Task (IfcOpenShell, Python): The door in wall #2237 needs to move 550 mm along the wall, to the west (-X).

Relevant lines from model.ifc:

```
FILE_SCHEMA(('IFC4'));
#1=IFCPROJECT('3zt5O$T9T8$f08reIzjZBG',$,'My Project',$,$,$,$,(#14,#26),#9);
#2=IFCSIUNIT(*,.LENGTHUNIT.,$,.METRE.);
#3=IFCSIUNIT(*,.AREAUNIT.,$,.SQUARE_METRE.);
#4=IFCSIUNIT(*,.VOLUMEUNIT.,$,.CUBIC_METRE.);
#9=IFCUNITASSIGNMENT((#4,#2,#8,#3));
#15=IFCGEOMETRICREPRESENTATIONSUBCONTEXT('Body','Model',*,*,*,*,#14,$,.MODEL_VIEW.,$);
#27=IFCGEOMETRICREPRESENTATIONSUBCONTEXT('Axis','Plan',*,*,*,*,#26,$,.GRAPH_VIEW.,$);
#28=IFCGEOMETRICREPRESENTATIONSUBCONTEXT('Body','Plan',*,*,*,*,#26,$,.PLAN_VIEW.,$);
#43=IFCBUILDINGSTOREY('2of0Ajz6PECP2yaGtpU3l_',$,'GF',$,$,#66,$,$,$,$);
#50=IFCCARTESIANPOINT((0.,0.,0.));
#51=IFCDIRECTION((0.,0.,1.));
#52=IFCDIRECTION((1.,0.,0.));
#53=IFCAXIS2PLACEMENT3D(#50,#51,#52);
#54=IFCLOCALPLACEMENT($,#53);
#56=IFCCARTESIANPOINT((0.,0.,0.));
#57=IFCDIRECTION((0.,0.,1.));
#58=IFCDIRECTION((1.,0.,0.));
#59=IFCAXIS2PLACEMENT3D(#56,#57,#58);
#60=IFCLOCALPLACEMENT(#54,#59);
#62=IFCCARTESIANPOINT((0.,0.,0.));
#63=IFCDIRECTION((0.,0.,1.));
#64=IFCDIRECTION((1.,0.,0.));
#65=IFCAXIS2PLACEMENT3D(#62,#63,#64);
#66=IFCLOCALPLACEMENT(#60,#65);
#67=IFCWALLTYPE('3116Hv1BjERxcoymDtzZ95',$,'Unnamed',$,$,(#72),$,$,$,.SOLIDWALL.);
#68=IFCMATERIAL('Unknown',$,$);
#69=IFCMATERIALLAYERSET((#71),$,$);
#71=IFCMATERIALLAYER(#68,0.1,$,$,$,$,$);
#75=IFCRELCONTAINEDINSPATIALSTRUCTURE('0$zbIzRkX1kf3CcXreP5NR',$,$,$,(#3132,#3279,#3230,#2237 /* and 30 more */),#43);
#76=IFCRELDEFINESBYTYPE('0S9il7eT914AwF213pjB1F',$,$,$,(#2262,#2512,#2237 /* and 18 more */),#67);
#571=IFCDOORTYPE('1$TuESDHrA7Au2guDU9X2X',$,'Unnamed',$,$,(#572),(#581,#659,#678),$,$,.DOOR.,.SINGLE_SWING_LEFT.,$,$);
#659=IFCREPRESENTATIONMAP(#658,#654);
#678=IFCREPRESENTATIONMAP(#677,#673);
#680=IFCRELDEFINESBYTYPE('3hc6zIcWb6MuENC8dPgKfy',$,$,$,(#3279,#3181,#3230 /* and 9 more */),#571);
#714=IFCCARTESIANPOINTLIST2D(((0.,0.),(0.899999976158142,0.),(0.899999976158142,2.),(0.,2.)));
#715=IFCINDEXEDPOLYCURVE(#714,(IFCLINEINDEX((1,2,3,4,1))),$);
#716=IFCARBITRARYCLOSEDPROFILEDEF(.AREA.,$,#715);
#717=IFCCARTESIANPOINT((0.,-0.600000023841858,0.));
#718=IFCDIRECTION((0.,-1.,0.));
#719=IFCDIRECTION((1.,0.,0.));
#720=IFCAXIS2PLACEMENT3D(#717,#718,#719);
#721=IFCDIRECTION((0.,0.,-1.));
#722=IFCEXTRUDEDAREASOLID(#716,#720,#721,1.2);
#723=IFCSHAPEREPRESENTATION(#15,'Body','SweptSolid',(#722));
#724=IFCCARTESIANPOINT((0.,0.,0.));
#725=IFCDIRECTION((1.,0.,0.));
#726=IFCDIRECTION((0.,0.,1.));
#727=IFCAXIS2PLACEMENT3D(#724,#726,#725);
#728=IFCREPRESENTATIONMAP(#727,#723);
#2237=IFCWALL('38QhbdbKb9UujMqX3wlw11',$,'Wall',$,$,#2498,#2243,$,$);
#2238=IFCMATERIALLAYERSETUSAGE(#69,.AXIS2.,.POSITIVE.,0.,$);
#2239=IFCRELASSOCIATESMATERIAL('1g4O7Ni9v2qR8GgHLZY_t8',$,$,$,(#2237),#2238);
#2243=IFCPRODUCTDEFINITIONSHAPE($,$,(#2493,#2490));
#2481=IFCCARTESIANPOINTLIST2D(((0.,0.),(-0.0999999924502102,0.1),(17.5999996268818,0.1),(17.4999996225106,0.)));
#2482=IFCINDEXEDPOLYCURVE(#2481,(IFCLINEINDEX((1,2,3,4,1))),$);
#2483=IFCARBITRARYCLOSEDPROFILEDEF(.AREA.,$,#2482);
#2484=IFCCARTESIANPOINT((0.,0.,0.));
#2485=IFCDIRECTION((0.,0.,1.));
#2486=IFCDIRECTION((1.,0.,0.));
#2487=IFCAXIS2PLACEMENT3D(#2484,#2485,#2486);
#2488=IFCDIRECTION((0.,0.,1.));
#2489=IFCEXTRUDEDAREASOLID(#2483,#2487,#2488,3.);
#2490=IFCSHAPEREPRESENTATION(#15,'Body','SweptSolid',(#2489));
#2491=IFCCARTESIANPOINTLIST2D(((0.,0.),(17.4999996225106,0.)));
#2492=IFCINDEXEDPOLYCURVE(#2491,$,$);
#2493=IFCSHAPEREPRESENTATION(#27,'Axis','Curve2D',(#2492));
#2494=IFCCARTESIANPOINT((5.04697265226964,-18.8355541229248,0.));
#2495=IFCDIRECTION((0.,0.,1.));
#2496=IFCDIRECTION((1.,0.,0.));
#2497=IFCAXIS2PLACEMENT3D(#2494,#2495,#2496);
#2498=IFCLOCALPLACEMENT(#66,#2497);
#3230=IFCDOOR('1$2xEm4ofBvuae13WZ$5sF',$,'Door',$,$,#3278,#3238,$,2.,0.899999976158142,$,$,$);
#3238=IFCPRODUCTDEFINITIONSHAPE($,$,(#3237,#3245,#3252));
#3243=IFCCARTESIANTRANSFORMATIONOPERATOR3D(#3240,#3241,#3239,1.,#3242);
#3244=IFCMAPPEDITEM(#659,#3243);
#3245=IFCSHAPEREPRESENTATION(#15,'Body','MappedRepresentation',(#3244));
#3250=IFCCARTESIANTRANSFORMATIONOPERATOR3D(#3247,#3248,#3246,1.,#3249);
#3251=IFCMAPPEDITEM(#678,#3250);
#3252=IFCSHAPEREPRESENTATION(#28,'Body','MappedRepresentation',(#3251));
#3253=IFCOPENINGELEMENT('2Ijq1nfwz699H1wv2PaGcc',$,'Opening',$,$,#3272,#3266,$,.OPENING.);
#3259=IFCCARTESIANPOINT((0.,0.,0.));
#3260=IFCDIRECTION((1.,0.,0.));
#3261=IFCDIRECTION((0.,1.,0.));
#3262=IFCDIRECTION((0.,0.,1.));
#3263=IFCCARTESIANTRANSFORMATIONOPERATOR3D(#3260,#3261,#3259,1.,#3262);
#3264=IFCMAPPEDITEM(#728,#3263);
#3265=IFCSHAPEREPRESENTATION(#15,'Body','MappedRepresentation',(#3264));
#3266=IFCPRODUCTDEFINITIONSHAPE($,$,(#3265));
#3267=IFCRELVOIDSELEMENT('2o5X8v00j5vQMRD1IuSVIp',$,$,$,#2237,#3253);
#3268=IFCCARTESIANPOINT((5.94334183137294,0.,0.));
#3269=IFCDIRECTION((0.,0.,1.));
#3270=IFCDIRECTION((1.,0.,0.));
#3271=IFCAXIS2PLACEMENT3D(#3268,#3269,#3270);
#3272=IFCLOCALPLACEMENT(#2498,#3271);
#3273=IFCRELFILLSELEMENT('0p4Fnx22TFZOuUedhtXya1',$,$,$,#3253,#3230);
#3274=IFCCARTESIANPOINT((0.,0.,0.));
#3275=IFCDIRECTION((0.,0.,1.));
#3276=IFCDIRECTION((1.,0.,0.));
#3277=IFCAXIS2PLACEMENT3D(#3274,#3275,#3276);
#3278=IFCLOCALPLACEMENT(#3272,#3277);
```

```python
import ifcopenshell
import ifcopenshell.api.geometry
import ifcopenshell.util.placement
import ifcopenshell.util.unit

model = ifcopenshell.open("model.ifc")
unit_scale = ifcopenshell.util.unit.calculate_unit_scale(model)

door = model.by_guid("1$2xEm4ofBvuae13WZ$5sF")
opening = door.FillsVoids[0].RelatingOpeningElement
wall = opening.VoidsElements[0].RelatingBuildingElement

wall_matrix = ifcopenshell.util.placement.get_local_placement(wall.ObjectPlacement)
shift = wall_matrix[:3, 0] * -0.55 / unit_scale
before = ifcopenshell.util.placement.get_local_placement(door.ObjectPlacement)[:3, 3].copy()

# The door is placed relative to its opening, so it follows when the opening moves.
matrix = ifcopenshell.util.placement.get_local_placement(opening.ObjectPlacement)
matrix[:3, 3] += shift
ifcopenshell.api.geometry.edit_object_placement(
    model, product=opening, matrix=matrix, is_si=False, should_transform_children=True
)

after = ifcopenshell.util.placement.get_local_placement(door.ObjectPlacement)[:3, 3]
print("door moved by", (after - before).round(3) + 0.0)

model.write("model-out.ifc")
```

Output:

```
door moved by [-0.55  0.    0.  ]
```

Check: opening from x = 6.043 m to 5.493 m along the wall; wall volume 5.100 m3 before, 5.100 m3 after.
